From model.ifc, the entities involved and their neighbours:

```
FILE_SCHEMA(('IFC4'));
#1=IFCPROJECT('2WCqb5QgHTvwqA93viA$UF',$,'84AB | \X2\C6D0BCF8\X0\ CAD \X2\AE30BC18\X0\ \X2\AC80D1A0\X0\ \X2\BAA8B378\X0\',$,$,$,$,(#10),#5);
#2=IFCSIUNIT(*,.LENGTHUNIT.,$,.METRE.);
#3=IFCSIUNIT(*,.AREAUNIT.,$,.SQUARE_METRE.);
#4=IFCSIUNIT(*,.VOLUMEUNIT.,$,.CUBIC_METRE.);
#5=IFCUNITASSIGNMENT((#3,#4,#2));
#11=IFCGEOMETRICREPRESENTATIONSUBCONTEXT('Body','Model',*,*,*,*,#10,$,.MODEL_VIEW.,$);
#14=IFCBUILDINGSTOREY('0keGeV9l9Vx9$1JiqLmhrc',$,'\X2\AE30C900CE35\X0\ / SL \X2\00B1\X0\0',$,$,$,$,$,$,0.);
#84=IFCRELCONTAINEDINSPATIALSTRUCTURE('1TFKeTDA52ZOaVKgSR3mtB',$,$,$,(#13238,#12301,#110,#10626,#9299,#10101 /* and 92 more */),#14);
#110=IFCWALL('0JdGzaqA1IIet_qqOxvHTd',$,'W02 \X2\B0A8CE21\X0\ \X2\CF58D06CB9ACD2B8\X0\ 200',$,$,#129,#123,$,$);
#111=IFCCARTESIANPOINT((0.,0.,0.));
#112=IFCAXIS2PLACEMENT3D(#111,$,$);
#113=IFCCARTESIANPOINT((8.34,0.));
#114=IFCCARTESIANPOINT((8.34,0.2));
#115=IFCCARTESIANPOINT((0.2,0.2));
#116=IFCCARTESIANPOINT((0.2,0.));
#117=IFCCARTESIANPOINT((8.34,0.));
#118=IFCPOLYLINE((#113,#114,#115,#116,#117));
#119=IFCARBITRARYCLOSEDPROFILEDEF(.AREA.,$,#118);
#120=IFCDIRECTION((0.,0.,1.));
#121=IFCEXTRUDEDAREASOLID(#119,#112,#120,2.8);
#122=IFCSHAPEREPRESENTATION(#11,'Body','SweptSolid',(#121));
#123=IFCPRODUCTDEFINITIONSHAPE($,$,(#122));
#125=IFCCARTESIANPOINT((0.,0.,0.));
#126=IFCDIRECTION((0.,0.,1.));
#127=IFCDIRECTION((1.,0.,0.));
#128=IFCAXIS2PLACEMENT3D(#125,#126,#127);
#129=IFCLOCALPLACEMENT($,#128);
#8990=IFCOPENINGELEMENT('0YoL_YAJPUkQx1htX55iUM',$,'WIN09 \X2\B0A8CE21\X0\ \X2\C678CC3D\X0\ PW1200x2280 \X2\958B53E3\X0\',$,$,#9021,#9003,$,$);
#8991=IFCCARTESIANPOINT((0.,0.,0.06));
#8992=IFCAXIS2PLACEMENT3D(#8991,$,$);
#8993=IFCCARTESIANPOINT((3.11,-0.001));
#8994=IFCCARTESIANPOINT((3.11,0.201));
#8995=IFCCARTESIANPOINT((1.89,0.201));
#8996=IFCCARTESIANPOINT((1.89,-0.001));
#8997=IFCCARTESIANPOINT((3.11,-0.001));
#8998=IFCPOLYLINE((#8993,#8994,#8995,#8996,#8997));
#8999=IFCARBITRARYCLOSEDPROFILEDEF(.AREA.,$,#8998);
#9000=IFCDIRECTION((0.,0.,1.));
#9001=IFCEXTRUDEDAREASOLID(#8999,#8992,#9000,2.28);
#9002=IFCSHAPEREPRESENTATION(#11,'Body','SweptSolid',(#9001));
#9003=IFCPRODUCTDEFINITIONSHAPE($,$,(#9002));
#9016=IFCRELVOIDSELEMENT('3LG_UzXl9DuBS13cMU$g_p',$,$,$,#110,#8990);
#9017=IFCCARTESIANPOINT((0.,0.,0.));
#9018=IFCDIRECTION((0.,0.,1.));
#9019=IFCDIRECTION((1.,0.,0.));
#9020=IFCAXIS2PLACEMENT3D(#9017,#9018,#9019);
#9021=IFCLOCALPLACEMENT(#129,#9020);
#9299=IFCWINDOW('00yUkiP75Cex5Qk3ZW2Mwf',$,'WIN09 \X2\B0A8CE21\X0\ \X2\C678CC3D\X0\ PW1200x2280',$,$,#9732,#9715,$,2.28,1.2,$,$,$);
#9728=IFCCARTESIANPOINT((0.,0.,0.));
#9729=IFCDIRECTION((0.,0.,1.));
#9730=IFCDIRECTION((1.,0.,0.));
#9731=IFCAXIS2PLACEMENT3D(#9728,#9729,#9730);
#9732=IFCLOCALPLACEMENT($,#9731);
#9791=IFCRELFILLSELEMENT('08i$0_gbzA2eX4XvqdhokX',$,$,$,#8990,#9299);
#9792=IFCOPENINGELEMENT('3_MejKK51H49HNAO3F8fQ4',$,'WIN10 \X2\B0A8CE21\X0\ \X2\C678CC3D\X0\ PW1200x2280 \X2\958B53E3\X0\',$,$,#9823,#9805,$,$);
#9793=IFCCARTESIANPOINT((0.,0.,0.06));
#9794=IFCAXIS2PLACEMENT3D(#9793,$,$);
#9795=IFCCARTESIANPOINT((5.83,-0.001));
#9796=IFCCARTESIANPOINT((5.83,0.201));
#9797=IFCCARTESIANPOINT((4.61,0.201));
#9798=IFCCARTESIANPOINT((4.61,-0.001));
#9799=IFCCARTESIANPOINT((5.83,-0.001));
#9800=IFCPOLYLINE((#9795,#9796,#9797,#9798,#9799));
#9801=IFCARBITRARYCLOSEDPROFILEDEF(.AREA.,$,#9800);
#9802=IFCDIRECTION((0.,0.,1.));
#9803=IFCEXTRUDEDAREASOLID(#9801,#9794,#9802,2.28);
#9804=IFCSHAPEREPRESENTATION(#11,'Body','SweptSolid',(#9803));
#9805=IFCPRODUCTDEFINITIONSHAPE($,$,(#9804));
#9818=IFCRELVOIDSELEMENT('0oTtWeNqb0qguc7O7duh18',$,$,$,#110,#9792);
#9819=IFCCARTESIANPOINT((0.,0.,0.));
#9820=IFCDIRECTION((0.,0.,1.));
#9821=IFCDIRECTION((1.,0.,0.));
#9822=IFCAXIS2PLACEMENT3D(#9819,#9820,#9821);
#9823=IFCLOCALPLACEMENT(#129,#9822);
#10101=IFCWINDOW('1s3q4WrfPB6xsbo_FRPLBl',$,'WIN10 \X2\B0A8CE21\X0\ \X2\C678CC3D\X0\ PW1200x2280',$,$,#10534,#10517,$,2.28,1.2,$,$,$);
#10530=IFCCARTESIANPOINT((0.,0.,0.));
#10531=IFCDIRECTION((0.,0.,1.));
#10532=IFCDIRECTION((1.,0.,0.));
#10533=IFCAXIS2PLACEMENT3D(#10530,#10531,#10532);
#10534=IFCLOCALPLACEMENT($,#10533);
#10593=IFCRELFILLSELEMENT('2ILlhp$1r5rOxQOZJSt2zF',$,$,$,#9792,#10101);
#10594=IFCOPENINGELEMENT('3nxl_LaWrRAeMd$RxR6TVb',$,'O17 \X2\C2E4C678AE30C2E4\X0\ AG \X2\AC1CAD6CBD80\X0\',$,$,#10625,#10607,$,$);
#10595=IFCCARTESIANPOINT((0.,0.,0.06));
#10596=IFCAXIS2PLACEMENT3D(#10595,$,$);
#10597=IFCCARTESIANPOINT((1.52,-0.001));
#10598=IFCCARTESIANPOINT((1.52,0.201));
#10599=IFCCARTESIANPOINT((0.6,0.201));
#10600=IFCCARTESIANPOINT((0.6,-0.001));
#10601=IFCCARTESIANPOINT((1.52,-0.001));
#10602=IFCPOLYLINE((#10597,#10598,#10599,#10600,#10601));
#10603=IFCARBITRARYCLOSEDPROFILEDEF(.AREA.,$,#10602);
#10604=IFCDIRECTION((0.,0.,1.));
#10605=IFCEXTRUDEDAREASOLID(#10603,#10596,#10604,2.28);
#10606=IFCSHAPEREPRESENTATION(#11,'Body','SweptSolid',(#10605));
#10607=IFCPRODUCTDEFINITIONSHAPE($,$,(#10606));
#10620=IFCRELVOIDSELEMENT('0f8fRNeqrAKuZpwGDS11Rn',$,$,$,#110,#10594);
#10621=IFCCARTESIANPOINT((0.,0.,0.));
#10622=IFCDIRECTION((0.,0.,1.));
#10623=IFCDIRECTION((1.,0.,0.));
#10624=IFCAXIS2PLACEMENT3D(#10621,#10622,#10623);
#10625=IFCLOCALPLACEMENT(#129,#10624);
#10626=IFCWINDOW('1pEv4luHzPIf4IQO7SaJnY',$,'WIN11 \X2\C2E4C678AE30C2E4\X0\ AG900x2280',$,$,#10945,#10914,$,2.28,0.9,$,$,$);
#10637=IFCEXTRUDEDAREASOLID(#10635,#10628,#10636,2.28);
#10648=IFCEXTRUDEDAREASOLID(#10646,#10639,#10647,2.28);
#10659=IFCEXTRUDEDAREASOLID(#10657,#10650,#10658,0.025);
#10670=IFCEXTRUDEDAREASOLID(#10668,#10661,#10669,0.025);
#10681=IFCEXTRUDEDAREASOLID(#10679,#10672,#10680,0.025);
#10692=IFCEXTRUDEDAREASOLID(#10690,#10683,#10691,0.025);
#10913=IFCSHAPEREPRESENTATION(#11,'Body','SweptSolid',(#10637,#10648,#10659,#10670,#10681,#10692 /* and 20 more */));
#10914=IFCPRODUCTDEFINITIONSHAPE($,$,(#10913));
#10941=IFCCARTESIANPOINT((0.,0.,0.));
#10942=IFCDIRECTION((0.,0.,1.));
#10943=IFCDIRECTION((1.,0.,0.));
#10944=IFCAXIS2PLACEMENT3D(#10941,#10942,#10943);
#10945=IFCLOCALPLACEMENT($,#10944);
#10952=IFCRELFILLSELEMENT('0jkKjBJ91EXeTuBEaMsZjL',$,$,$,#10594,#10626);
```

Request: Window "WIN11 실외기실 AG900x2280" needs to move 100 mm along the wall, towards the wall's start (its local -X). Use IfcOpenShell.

```python
import ifcopenshell
import ifcopenshell.api.geometry
import ifcopenshell.util.placement
import ifcopenshell.util.unit

model = ifcopenshell.open("model.ifc")
unit_scale = ifcopenshell.util.unit.calculate_unit_scale(model)

window = model.by_id(10626)
opening = window.FillsVoids[0].RelatingOpeningElement
wall = opening.VoidsElements[0].RelatingBuildingElement

wall_matrix = ifcopenshell.util.placement.get_local_placement(wall.ObjectPlacement)
shift = wall_matrix[:3, 0] * -0.1 / unit_scale
before = ifcopenshell.util.placement.get_local_placement(window.ObjectPlacement)[:3, 3].copy()

# The window is not placed relative to its opening, so move both.
for product in (opening, window):
    matrix = ifcopenshell.util.placement.get_local_placement(product.ObjectPlacement)
    matrix[:3, 3] += shift
    ifcopenshell.api.geometry.edit_object_placement(model, product=product, matrix=matrix, is_si=False)

after = ifcopenshell.util.placement.get_local_placement(window.ObjectPlacement)[:3, 3]
print("window moved by", (after - before).round(3) + 0.0)

model.write("model_updated.ifc")
```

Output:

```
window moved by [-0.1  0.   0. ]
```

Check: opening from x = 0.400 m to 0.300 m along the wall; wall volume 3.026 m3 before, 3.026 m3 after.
